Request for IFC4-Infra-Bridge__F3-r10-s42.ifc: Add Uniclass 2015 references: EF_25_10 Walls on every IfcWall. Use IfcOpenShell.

First a look at what the model holds.

```python
import ifcopenshell

model = ifcopenshell.open("IFC4-Infra-Bridge__F3-r10-s42.ifc")
print(model.schema)
print("classifications:", [c.Name for c in model.by_type("IfcClassification")])
for ifc_class in ("IfcDoor", "IfcRoof", "IfcStair", "IfcWall", "IfcWindow"):
    print(ifc_class, len(model.by_type(ifc_class)))
```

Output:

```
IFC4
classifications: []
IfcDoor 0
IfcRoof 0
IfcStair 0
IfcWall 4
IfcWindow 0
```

```python
import ifcopenshell
import ifcopenshell.api.classification

model = ifcopenshell.open("IFC4-Infra-Bridge__F3-r10-s42.ifc")

system = ifcopenshell.api.classification.add_classification(model, classification="Uniclass 2015")

codes = {
    "IfcWall": ("EF_25_10", "Walls"),
}
for ifc_class, (code, name) in codes.items():
    products = model.by_type(ifc_class)
    ifcopenshell.api.classification.add_reference(
        model, products=products, classification=system, identification=code, name=name
    )
    print(code, len(products))

model.write("IFC4-Infra-Bridge__F3-r10-s42-out.ifc")
```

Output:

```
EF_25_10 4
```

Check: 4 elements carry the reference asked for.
